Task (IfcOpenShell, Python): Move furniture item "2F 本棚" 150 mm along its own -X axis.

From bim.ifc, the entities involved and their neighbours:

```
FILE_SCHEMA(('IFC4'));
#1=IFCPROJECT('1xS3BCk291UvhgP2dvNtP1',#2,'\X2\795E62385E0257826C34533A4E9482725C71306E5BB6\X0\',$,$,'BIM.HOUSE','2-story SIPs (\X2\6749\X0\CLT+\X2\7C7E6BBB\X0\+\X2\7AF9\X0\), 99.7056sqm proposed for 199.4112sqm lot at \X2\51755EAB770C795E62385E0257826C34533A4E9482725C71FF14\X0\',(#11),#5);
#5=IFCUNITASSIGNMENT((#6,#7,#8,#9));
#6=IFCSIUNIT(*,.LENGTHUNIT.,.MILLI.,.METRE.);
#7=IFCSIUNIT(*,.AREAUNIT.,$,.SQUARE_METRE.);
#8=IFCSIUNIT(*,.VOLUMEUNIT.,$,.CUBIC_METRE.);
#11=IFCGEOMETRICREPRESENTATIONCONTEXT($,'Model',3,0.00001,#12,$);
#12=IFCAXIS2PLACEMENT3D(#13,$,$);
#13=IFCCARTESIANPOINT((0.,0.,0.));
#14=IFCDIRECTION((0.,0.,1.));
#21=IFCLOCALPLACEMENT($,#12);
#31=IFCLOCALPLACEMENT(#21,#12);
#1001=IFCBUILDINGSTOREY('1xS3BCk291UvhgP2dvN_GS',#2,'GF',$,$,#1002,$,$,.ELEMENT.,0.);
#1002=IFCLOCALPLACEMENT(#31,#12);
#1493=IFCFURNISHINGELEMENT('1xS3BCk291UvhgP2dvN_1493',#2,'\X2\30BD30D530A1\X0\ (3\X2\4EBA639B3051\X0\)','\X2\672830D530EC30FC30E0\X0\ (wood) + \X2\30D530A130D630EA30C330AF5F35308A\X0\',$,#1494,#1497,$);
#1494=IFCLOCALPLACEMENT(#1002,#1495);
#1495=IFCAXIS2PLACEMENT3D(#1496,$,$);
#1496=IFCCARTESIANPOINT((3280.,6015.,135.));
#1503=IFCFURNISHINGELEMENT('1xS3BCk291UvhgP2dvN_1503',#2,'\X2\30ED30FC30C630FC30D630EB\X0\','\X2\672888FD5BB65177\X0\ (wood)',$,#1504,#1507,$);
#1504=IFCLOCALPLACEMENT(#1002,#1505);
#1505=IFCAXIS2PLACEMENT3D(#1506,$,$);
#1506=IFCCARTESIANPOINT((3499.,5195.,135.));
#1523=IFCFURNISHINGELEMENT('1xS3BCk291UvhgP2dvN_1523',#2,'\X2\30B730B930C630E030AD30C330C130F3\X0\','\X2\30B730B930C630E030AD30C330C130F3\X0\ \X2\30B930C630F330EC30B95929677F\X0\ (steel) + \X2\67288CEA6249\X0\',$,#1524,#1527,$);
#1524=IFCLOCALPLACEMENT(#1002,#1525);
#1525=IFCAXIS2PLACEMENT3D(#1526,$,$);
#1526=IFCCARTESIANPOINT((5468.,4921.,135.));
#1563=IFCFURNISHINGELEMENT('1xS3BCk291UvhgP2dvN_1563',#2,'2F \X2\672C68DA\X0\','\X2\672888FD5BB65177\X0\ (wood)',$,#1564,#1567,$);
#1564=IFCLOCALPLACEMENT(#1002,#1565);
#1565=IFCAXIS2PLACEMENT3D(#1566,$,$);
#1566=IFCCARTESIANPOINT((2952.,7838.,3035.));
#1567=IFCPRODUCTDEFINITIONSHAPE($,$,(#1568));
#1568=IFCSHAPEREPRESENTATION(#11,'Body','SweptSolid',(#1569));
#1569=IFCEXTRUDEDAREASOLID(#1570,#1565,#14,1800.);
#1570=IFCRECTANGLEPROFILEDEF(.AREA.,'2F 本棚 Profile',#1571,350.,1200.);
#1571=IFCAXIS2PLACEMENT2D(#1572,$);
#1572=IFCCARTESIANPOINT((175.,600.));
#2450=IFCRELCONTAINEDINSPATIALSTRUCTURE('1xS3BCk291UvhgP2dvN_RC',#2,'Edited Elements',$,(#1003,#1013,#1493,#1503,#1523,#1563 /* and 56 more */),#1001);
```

```python
import ifcopenshell
import ifcopenshell.api.geometry
import ifcopenshell.util.placement
import ifcopenshell.util.unit

model = ifcopenshell.open("bim.ifc")
unit_scale = ifcopenshell.util.unit.calculate_unit_scale(model)

item = model.by_guid("1xS3BCk291UvhgP2dvN_1563")
matrix = ifcopenshell.util.placement.get_local_placement(item.ObjectPlacement)
matrix[:3, 3] -= matrix[:3, 0] * 0.15 / unit_scale
ifcopenshell.api.geometry.edit_object_placement(model, product=item, matrix=matrix, is_si=False)

print(ifcopenshell.util.placement.get_local_placement(item.ObjectPlacement).round(3) + 0.0)

model.write("bim-out.ifc")
```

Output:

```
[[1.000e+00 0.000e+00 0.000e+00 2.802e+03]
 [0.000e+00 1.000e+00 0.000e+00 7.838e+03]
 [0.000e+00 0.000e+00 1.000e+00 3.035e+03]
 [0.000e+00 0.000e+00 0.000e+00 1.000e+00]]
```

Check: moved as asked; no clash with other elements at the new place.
